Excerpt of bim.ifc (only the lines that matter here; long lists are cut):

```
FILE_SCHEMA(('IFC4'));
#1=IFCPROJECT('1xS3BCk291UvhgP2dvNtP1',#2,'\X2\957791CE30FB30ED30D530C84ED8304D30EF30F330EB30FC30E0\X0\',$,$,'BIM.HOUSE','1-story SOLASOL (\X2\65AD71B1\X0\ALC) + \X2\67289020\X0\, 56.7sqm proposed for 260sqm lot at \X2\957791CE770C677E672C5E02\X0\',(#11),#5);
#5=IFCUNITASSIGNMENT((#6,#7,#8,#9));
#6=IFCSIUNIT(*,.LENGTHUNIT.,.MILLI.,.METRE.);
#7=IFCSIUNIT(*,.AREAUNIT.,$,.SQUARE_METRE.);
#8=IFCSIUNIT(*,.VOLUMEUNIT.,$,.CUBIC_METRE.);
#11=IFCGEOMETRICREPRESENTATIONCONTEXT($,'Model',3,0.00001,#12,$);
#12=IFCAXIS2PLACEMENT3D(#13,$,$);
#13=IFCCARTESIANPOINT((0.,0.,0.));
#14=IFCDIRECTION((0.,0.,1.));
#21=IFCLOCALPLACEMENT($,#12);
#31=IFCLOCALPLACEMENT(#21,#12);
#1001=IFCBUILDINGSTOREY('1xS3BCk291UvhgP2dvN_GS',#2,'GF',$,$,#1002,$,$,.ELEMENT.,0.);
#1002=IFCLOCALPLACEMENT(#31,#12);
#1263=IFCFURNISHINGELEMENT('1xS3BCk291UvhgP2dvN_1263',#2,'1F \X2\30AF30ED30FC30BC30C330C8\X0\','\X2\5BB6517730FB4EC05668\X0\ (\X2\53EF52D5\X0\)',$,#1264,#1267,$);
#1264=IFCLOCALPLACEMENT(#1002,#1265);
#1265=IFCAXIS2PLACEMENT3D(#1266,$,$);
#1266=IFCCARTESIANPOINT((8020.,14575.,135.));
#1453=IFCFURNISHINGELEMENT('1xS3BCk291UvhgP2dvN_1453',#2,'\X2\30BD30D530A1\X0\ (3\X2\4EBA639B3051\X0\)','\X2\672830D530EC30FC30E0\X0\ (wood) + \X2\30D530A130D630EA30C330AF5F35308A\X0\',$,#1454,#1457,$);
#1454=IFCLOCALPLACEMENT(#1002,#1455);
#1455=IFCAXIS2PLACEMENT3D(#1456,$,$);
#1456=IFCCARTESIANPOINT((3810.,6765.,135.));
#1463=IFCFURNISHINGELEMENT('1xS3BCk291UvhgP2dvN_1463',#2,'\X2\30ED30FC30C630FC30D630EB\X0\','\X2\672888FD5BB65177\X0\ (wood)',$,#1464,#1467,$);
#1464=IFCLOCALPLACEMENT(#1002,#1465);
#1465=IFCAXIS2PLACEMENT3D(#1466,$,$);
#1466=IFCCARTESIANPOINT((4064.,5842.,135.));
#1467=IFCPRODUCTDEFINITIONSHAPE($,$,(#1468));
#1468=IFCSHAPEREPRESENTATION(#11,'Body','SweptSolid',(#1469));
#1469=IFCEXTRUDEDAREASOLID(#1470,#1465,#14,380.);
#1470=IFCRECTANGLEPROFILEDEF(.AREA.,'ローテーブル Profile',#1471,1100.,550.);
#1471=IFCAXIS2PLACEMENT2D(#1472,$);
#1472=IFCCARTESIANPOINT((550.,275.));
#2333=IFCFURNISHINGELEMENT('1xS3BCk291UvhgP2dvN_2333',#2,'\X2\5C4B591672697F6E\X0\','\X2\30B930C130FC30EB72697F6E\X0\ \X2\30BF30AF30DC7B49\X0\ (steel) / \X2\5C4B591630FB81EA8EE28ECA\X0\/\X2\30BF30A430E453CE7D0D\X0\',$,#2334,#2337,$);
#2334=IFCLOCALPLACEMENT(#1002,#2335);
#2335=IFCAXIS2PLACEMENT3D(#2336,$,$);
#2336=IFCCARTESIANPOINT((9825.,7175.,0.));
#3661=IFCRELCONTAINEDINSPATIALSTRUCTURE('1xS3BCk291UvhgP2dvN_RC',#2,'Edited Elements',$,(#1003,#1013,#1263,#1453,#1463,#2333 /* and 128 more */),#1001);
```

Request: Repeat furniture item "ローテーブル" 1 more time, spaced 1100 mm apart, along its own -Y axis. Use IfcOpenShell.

```python
import ifcopenshell
import ifcopenshell.api.geometry
import ifcopenshell.api.root
import ifcopenshell.util.element
import ifcopenshell.util.placement
import ifcopenshell.util.unit

model = ifcopenshell.open("bim.ifc")
unit_scale = ifcopenshell.util.unit.calculate_unit_scale(model)


def reuse_history(source, copy):
    """copy_class also copies each property set's owner history, people and application; keep the originals."""
    for rel in copy.IsDefinedBy:
        if rel.is_a("IfcRelDefinesByProperties") and (history := rel.RelatingPropertyDefinition.OwnerHistory):
            rel.RelatingPropertyDefinition.OwnerHistory = source.OwnerHistory
            ifcopenshell.util.element.remove_deep2(model, history)


source = model.by_guid("1xS3BCk291UvhgP2dvN_1463")
base = ifcopenshell.util.placement.get_local_placement(source.ObjectPlacement)
step = -base[:3, 1] * 1.1 / unit_scale

for i in range(1, 2):
    copy = ifcopenshell.api.root.copy_class(model, product=source)
    copy.Representation = ifcopenshell.util.element.copy_deep(
        model, source.Representation, exclude=["IfcGeometricRepresentationContext", "IfcRepresentationMap"]
    )
    reuse_history(source, copy)
    matrix = base.copy()
    matrix[:3, 3] += i * step
    print("added at", matrix[:3, 3].round(3) + 0.0)
    ifcopenshell.api.geometry.edit_object_placement(model, product=copy, matrix=matrix, is_si=False)

model.write("bim_updated.ifc")
```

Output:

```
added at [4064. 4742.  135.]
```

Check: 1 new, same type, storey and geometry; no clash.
